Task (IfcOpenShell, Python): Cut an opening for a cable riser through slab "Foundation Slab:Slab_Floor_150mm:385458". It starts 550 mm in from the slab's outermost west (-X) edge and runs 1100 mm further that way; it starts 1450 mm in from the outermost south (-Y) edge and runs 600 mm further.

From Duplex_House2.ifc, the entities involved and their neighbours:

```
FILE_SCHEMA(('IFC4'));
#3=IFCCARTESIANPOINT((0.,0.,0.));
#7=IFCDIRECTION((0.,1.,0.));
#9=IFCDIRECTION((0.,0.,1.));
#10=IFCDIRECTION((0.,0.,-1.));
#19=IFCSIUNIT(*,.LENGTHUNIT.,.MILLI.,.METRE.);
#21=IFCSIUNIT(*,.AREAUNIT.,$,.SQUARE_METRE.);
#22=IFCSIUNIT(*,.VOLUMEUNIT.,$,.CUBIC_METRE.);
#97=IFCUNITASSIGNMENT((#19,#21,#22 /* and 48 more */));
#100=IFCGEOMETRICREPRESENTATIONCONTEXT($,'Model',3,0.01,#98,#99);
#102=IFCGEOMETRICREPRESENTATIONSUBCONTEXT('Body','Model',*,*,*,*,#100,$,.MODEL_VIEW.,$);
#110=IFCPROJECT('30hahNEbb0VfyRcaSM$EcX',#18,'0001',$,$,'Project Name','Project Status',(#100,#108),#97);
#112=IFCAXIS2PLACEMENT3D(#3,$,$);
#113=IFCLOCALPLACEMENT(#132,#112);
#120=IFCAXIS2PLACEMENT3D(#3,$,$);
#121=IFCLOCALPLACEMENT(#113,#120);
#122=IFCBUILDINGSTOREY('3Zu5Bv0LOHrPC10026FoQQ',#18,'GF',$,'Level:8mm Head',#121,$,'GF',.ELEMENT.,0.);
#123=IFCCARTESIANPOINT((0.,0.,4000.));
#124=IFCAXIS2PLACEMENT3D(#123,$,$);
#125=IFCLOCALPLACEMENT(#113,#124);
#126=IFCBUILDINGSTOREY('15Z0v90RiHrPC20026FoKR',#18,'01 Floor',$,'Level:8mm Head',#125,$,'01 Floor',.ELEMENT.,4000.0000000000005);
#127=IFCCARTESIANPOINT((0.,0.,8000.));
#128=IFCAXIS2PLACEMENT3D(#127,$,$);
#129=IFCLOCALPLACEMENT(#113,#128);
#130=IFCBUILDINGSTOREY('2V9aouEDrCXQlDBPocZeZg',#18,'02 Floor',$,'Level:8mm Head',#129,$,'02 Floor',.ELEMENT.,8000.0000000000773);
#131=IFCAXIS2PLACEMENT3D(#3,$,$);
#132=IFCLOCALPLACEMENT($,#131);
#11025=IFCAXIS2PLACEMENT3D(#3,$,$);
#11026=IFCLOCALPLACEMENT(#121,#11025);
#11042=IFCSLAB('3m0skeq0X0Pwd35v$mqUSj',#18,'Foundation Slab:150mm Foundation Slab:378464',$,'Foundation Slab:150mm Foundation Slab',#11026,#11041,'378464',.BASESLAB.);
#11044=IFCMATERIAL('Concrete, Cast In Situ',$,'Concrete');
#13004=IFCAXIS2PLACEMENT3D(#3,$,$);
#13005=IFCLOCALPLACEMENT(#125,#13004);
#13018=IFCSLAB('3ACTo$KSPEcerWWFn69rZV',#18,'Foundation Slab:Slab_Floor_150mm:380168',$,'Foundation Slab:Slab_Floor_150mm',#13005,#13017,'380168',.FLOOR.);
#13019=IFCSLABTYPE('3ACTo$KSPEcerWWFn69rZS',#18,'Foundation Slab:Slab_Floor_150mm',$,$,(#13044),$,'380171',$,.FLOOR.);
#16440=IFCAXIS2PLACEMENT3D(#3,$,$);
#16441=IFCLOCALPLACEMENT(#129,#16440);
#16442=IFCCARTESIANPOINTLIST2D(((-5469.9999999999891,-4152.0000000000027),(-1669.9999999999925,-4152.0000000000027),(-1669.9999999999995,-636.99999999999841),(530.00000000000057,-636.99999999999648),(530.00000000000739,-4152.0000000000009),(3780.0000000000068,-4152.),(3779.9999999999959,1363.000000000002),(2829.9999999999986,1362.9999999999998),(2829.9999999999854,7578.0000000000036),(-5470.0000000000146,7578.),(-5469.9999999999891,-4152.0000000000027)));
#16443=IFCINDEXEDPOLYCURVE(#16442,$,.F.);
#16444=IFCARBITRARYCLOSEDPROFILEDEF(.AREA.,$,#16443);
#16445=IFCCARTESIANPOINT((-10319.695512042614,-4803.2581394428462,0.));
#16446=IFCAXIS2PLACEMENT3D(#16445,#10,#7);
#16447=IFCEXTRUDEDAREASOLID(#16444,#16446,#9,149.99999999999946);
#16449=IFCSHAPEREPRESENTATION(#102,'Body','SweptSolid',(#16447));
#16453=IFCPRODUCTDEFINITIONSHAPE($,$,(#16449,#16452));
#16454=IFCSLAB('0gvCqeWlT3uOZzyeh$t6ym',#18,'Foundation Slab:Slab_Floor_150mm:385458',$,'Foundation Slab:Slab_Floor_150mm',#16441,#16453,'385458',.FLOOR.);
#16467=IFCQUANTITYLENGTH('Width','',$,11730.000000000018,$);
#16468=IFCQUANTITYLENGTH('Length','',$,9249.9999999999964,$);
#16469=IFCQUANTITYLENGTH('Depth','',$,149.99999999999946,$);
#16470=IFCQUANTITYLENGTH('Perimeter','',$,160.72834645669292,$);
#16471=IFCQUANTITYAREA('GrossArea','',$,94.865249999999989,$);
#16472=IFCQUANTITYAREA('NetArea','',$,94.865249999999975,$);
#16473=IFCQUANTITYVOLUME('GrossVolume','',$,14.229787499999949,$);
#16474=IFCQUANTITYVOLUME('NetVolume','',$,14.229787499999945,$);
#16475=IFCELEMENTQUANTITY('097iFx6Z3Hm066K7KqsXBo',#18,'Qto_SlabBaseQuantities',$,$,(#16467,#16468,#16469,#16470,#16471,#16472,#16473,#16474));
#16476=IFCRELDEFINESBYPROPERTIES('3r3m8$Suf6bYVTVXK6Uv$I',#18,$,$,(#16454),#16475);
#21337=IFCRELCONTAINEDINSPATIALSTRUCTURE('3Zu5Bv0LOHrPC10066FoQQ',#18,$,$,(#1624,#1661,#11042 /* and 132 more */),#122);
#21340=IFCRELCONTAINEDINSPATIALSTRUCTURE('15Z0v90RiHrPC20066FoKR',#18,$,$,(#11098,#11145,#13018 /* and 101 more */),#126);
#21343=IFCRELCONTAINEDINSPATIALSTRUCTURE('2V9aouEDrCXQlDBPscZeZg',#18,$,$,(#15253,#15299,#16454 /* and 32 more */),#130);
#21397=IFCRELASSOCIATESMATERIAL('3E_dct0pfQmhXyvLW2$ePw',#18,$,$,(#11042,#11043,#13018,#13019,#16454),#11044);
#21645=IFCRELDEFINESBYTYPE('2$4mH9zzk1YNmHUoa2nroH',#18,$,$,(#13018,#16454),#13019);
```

```python
import numpy as np
import ifcopenshell
import ifcopenshell.api.feature
import ifcopenshell.api.geometry
import ifcopenshell.api.pset
import ifcopenshell.api.root
import ifcopenshell.geom
import ifcopenshell.util.element
import ifcopenshell.util.placement
import ifcopenshell.util.representation
import ifcopenshell.util.shape
import ifcopenshell.util.unit

model = ifcopenshell.open("Duplex_House2.ifc")
unit_scale = ifcopenshell.util.unit.calculate_unit_scale(model)
area_scale = ifcopenshell.util.unit.calculate_unit_scale(model, "AREAUNIT")
volume_scale = ifcopenshell.util.unit.calculate_unit_scale(model, "VOLUMEUNIT")
settings = ifcopenshell.geom.settings()


def volume(element):
    """Net volume in cubic metres, openings subtracted."""
    shape = ifcopenshell.geom.create_shape(settings, element)
    return ifcopenshell.util.shape.get_volume(shape.geometry)


slab = model.by_guid("0gvCqeWlT3uOZzyeh$t6ym")
before = volume(slab)

# Extent in the slab's own axes, in metres. The edges named are its -X and -Y sides.
slab_shape = ifcopenshell.geom.create_shape(settings, slab)
vertices = ifcopenshell.util.shape.get_vertices(slab_shape.geometry)
x_min, y_min, bottom = vertices.min(axis=0)
top = vertices[:, 2].max()

opening = ifcopenshell.api.root.create_entity(model, ifc_class="IfcOpeningElement", name="Cable riser opening", predefined_type="OPENING")
context = ifcopenshell.util.representation.get_context(model, "Model", "Body", "MODEL_VIEW")
width, depth = 1.1, 0.6
outline = [(0.0, 0.0), (width, 0.0), (width, depth), (0.0, depth), (0.0, 0.0)]
# Overshoot both faces by 50 mm so the cut is clean.
shape = ifcopenshell.api.geometry.add_slab_representation(
    model, context=context, depth=top - bottom + 0.1, polyline=outline
)
ifcopenshell.api.geometry.assign_representation(model, product=opening, representation=shape)

matrix = ifcopenshell.util.placement.get_local_placement(slab.ObjectPlacement)
matrix[:, 3] = matrix @ np.append(np.array([x_min + 0.55, y_min + 1.45, bottom - 0.05]) / unit_scale, 1.0)
ifcopenshell.api.geometry.edit_object_placement(model, product=opening, matrix=matrix, is_si=False)
ifcopenshell.api.feature.add_feature(model, feature=opening, element=slab)

after = volume(slab)

# Update the slab's stored quantities.
qto = model.by_id(ifcopenshell.util.element.get_pset(slab, "Qto_SlabBaseQuantities", should_inherit=False)["id"])
ifcopenshell.api.pset.edit_qto(model, qto=qto, properties={
    "NetArea": after / (top - bottom) / area_scale,
    "NetVolume": after / volume_scale,
})

print(f"slab volume {before:.3f} -> {after:.3f} m3")

model.write("Duplex_House2_v2.ifc")
```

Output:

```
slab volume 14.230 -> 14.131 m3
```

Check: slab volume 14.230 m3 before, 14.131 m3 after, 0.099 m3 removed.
